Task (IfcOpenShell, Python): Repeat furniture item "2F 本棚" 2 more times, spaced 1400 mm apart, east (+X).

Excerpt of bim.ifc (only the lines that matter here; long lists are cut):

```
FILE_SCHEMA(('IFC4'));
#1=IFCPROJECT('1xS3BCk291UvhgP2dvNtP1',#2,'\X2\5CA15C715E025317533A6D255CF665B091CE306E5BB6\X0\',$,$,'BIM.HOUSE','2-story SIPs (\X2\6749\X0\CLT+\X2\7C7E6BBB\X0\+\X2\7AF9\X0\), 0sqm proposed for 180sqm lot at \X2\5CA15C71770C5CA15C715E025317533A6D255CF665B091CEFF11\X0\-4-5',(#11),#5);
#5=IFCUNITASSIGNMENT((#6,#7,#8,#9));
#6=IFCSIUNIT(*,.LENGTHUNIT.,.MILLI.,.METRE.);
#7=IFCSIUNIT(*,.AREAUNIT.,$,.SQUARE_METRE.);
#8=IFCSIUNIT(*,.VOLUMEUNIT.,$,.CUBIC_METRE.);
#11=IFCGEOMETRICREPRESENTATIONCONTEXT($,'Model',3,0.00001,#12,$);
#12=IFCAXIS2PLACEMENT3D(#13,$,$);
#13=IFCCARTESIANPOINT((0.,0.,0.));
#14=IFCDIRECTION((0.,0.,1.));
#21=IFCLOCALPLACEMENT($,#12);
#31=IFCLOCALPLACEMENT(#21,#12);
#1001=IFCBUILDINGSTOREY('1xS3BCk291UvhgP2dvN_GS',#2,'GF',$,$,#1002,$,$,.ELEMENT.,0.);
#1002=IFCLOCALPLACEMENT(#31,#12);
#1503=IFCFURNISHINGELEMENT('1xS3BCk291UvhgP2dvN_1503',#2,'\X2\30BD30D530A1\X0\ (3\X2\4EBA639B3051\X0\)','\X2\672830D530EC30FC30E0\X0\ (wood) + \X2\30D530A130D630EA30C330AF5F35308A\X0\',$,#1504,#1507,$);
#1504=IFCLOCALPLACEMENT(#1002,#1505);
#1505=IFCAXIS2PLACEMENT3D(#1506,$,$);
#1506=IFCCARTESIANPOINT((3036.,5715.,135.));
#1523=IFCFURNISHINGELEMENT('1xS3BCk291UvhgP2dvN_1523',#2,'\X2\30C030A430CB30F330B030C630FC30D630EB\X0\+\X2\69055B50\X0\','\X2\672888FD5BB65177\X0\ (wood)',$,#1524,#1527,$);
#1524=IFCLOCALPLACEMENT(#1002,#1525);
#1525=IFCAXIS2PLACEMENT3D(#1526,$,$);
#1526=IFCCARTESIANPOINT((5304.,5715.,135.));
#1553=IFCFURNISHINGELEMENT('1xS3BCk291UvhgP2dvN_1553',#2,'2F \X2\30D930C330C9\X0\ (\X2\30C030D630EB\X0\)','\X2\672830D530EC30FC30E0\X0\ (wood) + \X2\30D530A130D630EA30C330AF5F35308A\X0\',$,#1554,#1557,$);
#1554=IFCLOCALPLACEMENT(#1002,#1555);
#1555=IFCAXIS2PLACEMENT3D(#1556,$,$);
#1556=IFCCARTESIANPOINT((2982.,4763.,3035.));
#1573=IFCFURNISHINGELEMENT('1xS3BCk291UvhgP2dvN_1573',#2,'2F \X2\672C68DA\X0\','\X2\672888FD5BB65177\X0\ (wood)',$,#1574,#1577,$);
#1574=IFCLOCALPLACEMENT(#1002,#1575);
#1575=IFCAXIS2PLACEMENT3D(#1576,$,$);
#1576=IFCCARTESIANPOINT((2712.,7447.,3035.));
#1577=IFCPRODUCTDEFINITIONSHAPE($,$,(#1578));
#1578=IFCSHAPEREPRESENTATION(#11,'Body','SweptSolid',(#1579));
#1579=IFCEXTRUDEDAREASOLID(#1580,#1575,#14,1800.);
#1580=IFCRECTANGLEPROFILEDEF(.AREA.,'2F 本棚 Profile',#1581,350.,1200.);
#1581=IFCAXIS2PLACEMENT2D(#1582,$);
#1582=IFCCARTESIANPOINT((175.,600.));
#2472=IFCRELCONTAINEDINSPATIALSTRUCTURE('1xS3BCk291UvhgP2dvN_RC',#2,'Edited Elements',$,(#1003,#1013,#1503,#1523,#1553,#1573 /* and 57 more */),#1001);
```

```python
import numpy as np
import ifcopenshell
import ifcopenshell.api.geometry
import ifcopenshell.api.root
import ifcopenshell.util.element
import ifcopenshell.util.placement

model = ifcopenshell.open("bim.ifc")


def reuse_history(source, copy):
    """copy_class also copies each property set's owner history, people and application; keep the originals."""
    for rel in copy.IsDefinedBy:
        if rel.is_a("IfcRelDefinesByProperties") and (history := rel.RelatingPropertyDefinition.OwnerHistory):
            rel.RelatingPropertyDefinition.OwnerHistory = source.OwnerHistory
            ifcopenshell.util.element.remove_deep2(model, history)


source = model.by_guid("1xS3BCk291UvhgP2dvN_1573")
base = ifcopenshell.util.placement.get_local_placement(source.ObjectPlacement)
step = np.array([1.0, 0.0, 0.0]) * 1400.0

for i in range(1, 3):
    copy = ifcopenshell.api.root.copy_class(model, product=source)
    copy.Representation = ifcopenshell.util.element.copy_deep(
        model, source.Representation, exclude=["IfcGeometricRepresentationContext", "IfcRepresentationMap"]
    )
    reuse_history(source, copy)
    matrix = base.copy()
    matrix[:3, 3] += i * step
    print("added at", matrix[:3, 3].round(3) + 0.0)
    ifcopenshell.api.geometry.edit_object_placement(model, product=copy, matrix=matrix, is_si=False)

model.write("bim_rev.ifc")
```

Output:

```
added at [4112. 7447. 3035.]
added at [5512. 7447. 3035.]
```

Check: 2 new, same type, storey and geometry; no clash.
